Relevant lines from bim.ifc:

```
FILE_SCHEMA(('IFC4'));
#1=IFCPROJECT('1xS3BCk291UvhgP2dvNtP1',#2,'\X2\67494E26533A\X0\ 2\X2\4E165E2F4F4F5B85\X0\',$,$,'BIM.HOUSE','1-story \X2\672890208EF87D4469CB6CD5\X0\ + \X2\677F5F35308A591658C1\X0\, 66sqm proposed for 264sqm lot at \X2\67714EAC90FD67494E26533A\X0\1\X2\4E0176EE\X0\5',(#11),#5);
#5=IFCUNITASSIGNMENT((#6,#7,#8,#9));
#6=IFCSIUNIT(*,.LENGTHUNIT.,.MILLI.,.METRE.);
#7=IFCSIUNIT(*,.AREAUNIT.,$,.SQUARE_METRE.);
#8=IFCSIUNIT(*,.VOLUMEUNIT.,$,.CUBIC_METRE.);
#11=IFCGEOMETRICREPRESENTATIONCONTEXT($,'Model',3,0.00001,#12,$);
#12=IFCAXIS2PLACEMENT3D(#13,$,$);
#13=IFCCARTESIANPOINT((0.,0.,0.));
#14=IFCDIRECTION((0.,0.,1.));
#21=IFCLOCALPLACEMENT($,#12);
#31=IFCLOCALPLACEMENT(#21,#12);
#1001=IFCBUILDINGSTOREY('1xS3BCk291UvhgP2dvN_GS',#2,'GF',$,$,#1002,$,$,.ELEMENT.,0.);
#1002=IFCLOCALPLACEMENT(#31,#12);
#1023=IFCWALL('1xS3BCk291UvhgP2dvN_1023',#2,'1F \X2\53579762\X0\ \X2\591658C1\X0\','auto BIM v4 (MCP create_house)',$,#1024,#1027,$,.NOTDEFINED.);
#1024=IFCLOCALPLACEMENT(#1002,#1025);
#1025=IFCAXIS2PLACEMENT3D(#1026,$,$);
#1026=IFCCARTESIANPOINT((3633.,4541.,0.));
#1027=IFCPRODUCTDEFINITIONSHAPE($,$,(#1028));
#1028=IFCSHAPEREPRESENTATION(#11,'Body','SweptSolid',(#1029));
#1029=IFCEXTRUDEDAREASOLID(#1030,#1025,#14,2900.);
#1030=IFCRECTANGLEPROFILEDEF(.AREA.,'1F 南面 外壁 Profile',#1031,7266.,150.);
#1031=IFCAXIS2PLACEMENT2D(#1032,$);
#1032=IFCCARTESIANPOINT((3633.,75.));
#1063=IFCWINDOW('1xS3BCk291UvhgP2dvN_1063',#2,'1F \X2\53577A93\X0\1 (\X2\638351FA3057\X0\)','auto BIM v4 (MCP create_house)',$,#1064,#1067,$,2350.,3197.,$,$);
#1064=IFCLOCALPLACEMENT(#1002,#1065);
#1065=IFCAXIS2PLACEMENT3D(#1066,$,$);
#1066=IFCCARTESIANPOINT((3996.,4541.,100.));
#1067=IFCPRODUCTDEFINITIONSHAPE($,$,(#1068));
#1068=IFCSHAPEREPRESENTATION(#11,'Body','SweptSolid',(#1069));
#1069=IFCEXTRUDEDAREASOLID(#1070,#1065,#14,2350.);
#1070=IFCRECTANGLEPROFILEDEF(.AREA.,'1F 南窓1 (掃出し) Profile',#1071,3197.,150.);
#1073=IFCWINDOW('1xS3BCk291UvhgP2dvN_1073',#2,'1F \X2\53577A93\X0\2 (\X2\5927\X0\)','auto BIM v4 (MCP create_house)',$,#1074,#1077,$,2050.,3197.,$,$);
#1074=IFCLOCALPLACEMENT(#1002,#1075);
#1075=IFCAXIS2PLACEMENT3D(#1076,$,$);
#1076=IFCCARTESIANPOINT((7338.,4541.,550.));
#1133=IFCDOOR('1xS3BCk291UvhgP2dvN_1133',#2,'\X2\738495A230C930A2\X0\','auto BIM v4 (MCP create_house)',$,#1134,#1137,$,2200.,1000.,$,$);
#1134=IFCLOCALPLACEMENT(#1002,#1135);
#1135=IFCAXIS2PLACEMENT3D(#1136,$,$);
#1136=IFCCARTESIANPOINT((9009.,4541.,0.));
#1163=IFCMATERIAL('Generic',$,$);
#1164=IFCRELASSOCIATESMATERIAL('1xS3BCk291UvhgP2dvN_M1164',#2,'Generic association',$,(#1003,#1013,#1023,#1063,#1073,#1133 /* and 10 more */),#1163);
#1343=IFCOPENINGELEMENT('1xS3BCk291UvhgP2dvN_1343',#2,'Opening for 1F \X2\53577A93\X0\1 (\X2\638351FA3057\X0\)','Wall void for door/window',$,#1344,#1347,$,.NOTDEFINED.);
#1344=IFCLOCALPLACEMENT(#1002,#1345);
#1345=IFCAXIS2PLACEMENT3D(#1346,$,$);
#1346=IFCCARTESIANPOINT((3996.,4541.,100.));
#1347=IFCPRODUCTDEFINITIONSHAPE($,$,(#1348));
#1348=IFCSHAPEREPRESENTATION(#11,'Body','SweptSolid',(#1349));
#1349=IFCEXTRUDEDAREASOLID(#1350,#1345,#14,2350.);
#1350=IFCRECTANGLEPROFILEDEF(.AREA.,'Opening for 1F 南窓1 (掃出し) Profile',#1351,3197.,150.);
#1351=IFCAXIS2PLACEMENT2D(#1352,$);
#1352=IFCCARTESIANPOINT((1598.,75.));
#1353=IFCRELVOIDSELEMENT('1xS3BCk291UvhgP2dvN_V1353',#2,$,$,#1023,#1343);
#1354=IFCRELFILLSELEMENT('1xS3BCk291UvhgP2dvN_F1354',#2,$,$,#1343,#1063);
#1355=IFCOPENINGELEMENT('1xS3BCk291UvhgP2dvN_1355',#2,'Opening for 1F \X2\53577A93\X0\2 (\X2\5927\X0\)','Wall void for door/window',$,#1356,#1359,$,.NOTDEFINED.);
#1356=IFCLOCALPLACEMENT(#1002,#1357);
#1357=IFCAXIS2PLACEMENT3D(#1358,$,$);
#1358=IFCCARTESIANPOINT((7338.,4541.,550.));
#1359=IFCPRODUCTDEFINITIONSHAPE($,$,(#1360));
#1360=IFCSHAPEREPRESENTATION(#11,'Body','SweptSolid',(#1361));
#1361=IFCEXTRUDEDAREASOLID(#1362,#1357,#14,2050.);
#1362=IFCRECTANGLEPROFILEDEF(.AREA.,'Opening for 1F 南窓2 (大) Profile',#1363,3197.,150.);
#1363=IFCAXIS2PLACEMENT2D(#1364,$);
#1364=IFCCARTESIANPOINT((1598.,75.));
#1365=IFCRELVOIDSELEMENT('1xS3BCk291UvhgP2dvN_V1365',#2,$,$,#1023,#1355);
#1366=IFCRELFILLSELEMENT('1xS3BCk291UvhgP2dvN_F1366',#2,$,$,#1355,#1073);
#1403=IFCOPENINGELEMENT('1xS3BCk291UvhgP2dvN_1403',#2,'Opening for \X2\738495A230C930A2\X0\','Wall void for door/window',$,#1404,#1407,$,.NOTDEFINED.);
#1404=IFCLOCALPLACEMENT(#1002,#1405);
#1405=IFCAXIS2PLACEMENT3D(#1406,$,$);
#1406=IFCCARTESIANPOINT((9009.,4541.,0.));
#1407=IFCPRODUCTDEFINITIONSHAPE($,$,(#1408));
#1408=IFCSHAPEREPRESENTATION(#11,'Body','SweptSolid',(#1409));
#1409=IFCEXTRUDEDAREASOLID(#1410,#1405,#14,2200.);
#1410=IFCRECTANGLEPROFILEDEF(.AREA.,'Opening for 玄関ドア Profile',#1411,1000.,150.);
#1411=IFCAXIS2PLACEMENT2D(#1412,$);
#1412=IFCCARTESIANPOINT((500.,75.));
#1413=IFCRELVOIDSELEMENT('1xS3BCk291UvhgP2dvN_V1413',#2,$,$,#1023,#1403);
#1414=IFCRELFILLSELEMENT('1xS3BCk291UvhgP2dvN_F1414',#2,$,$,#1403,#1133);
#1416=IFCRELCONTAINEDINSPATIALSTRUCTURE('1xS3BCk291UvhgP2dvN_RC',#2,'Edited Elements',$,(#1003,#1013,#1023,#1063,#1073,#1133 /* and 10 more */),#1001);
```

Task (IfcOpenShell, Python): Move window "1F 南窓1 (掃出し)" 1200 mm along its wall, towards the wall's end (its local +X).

```python
import ifcopenshell
import ifcopenshell.api.geometry
import ifcopenshell.util.placement
import ifcopenshell.util.unit

model = ifcopenshell.open("bim.ifc")
unit_scale = ifcopenshell.util.unit.calculate_unit_scale(model)

window = model.by_guid("1xS3BCk291UvhgP2dvN_1063")
opening = window.FillsVoids[0].RelatingOpeningElement
wall = opening.VoidsElements[0].RelatingBuildingElement

wall_matrix = ifcopenshell.util.placement.get_local_placement(wall.ObjectPlacement)
shift = wall_matrix[:3, 0] * 1.2 / unit_scale
before = ifcopenshell.util.placement.get_local_placement(window.ObjectPlacement)[:3, 3].copy()

# The window is not placed relative to its opening, so move both.
for product in (opening, window):
    matrix = ifcopenshell.util.placement.get_local_placement(product.ObjectPlacement)
    matrix[:3, 3] += shift
    ifcopenshell.api.geometry.edit_object_placement(model, product=product, matrix=matrix, is_si=False)

after = ifcopenshell.util.placement.get_local_placement(window.ObjectPlacement)[:3, 3]
print("window moved by", (after - before).round(3) + 0.0)

model.write("bim-out.ifc")
```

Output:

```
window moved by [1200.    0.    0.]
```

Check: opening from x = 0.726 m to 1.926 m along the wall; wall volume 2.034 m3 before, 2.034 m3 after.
